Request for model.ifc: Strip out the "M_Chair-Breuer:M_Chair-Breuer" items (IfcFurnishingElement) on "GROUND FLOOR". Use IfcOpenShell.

First a look at what the model holds.

```python
import ifcopenshell
import ifcopenshell.util.element

model = ifcopenshell.open("model.ifc")
print(model.schema)
storey = next(s for s in model.by_type("IfcBuildingStorey") if s.Name == "GROUND FLOOR")
furniture = [e for e in ifcopenshell.util.element.get_decomposition(storey) if e.is_a("IfcFurnishingElement")]
seen = {}
for e in furniture:
    element_type = ifcopenshell.util.element.get_type(e)
    name = element_type.Name if element_type not in (None, e) else None
    seen[name] = seen.get(name, 0) + 1
for name, count in sorted(seen.items(), key=str):
    print(count, "x", name)
```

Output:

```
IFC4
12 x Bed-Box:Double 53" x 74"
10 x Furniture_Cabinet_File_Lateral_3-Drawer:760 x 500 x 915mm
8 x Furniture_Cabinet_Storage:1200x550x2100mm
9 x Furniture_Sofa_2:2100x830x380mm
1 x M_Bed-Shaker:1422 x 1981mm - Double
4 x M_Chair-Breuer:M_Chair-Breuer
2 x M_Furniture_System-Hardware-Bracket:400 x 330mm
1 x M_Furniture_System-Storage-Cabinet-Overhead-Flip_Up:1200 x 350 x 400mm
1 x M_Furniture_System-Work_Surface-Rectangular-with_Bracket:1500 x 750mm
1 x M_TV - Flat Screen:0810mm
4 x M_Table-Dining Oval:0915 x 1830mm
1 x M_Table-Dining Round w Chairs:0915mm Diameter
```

```python
import ifcopenshell
import ifcopenshell.api.root
import ifcopenshell.util.element

model = ifcopenshell.open("model.ifc")

storey = next(s for s in model.by_type("IfcBuildingStorey") if s.Name == "GROUND FLOOR")
furniture = [e for e in ifcopenshell.util.element.get_decomposition(storey) if e.is_a("IfcFurnishingElement")]
targets = [e for e in furniture if (t := ifcopenshell.util.element.get_type(e)) not in (None, e) and t.Name == "M_Chair-Breuer:M_Chair-Breuer"]

for e in targets:
    ifcopenshell.api.root.remove_product(model, product=e)
print(len(targets), "removed")

model.write("model-out.ifc")
```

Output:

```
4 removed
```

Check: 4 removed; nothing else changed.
